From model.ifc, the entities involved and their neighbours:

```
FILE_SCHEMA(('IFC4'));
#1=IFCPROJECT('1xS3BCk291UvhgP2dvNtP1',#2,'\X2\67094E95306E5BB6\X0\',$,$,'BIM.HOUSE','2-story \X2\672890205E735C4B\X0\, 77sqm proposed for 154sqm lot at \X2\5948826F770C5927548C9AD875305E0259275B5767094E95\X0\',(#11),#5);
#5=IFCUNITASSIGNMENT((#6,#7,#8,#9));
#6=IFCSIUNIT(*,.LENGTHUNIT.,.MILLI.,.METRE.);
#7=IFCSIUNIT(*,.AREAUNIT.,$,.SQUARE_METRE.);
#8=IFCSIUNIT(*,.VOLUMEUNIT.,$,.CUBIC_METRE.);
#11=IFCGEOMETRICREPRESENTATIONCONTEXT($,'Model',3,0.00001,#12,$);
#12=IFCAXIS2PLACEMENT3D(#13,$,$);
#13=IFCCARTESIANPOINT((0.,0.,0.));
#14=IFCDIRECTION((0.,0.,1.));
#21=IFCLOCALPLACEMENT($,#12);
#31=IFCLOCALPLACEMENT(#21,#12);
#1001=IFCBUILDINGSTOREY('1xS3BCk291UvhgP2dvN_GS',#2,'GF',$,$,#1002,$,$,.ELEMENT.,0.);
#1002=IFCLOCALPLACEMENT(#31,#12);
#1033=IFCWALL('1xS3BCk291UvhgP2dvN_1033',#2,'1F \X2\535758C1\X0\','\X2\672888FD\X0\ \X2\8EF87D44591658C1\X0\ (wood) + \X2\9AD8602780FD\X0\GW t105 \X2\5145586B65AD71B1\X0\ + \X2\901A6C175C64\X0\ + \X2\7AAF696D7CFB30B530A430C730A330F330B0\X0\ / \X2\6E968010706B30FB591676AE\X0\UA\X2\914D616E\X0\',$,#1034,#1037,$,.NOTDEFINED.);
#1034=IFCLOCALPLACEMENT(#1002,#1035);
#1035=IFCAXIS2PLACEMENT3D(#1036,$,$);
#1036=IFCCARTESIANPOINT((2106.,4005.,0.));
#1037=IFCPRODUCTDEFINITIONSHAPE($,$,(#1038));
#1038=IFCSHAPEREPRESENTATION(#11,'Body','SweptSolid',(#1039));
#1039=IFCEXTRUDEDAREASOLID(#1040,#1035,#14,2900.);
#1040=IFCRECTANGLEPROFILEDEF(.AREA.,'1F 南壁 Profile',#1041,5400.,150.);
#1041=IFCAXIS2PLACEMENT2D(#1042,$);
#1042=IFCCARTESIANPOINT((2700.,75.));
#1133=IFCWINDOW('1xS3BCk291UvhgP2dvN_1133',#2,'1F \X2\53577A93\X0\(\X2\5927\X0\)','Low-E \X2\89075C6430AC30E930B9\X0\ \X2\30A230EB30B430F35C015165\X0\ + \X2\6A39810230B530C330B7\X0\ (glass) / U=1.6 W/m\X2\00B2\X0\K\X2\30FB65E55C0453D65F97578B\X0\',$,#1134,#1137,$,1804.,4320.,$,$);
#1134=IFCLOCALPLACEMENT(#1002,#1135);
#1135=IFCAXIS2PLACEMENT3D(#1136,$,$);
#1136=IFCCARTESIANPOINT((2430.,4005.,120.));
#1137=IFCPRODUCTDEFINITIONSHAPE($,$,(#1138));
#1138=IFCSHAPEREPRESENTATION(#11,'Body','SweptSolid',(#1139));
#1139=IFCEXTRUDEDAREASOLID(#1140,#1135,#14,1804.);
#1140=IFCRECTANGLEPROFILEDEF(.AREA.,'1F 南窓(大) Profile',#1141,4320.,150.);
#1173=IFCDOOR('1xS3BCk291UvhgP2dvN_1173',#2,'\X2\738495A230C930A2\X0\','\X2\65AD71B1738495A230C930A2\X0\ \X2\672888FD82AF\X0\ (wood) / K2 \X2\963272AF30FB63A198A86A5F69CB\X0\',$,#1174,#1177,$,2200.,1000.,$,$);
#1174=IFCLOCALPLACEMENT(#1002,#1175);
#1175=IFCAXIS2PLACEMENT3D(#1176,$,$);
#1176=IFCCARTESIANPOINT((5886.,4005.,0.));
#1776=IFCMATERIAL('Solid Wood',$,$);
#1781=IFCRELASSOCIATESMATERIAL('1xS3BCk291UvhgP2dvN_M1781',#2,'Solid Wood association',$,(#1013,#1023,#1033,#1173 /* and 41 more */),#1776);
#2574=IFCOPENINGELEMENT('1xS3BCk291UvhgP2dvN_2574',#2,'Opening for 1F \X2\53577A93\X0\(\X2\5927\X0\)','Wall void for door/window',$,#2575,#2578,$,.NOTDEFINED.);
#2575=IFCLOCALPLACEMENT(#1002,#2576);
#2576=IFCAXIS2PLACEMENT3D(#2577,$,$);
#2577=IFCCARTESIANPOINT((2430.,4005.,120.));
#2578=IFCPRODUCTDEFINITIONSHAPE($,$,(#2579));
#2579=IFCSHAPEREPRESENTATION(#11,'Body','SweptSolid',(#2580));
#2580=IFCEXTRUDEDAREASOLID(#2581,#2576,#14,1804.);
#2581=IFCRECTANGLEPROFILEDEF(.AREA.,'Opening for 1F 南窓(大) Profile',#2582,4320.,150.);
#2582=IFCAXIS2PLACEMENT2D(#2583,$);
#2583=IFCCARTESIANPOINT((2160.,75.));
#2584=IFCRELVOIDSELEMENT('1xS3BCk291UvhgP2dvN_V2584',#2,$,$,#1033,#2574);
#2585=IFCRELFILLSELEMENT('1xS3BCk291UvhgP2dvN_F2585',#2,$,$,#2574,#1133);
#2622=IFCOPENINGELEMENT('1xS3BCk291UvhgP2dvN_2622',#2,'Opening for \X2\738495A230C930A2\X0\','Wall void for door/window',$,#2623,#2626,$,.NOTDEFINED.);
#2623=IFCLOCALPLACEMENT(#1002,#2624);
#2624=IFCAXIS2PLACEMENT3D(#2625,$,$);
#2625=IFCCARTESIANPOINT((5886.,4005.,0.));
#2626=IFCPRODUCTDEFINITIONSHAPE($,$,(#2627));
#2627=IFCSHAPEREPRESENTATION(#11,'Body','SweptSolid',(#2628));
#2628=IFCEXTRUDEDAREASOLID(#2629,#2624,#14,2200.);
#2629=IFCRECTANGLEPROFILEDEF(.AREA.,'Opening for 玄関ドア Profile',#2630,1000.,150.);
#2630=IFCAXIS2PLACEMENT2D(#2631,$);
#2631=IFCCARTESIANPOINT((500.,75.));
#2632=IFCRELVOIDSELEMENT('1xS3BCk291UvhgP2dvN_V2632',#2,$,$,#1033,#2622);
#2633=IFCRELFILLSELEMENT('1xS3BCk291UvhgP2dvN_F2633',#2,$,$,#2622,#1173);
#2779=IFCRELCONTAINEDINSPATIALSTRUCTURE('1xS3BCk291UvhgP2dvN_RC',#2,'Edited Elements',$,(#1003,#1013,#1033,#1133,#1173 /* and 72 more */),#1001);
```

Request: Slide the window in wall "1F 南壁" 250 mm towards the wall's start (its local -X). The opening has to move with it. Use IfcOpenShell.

```python
import ifcopenshell
import ifcopenshell.api.geometry
import ifcopenshell.util.placement

model = ifcopenshell.open("model.ifc")

window = model.by_id(1133)
opening = window.FillsVoids[0].RelatingOpeningElement
wall = opening.VoidsElements[0].RelatingBuildingElement

wall_matrix = ifcopenshell.util.placement.get_local_placement(wall.ObjectPlacement)
shift = wall_matrix[:3, 0] * -250.0
before = ifcopenshell.util.placement.get_local_placement(window.ObjectPlacement)[:3, 3].copy()

# The window is not placed relative to its opening, so move both.
for product in (opening, window):
    matrix = ifcopenshell.util.placement.get_local_placement(product.ObjectPlacement)
    matrix[:3, 3] += shift
    ifcopenshell.api.geometry.edit_object_placement(model, product=product, matrix=matrix, is_si=False)

after = ifcopenshell.util.placement.get_local_placement(window.ObjectPlacement)[:3, 3]
print("window moved by", (after - before).round(3) + 0.0)

model.write("model-out.ifc")
```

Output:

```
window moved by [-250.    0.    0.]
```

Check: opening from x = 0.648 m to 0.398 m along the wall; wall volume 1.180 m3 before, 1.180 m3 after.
